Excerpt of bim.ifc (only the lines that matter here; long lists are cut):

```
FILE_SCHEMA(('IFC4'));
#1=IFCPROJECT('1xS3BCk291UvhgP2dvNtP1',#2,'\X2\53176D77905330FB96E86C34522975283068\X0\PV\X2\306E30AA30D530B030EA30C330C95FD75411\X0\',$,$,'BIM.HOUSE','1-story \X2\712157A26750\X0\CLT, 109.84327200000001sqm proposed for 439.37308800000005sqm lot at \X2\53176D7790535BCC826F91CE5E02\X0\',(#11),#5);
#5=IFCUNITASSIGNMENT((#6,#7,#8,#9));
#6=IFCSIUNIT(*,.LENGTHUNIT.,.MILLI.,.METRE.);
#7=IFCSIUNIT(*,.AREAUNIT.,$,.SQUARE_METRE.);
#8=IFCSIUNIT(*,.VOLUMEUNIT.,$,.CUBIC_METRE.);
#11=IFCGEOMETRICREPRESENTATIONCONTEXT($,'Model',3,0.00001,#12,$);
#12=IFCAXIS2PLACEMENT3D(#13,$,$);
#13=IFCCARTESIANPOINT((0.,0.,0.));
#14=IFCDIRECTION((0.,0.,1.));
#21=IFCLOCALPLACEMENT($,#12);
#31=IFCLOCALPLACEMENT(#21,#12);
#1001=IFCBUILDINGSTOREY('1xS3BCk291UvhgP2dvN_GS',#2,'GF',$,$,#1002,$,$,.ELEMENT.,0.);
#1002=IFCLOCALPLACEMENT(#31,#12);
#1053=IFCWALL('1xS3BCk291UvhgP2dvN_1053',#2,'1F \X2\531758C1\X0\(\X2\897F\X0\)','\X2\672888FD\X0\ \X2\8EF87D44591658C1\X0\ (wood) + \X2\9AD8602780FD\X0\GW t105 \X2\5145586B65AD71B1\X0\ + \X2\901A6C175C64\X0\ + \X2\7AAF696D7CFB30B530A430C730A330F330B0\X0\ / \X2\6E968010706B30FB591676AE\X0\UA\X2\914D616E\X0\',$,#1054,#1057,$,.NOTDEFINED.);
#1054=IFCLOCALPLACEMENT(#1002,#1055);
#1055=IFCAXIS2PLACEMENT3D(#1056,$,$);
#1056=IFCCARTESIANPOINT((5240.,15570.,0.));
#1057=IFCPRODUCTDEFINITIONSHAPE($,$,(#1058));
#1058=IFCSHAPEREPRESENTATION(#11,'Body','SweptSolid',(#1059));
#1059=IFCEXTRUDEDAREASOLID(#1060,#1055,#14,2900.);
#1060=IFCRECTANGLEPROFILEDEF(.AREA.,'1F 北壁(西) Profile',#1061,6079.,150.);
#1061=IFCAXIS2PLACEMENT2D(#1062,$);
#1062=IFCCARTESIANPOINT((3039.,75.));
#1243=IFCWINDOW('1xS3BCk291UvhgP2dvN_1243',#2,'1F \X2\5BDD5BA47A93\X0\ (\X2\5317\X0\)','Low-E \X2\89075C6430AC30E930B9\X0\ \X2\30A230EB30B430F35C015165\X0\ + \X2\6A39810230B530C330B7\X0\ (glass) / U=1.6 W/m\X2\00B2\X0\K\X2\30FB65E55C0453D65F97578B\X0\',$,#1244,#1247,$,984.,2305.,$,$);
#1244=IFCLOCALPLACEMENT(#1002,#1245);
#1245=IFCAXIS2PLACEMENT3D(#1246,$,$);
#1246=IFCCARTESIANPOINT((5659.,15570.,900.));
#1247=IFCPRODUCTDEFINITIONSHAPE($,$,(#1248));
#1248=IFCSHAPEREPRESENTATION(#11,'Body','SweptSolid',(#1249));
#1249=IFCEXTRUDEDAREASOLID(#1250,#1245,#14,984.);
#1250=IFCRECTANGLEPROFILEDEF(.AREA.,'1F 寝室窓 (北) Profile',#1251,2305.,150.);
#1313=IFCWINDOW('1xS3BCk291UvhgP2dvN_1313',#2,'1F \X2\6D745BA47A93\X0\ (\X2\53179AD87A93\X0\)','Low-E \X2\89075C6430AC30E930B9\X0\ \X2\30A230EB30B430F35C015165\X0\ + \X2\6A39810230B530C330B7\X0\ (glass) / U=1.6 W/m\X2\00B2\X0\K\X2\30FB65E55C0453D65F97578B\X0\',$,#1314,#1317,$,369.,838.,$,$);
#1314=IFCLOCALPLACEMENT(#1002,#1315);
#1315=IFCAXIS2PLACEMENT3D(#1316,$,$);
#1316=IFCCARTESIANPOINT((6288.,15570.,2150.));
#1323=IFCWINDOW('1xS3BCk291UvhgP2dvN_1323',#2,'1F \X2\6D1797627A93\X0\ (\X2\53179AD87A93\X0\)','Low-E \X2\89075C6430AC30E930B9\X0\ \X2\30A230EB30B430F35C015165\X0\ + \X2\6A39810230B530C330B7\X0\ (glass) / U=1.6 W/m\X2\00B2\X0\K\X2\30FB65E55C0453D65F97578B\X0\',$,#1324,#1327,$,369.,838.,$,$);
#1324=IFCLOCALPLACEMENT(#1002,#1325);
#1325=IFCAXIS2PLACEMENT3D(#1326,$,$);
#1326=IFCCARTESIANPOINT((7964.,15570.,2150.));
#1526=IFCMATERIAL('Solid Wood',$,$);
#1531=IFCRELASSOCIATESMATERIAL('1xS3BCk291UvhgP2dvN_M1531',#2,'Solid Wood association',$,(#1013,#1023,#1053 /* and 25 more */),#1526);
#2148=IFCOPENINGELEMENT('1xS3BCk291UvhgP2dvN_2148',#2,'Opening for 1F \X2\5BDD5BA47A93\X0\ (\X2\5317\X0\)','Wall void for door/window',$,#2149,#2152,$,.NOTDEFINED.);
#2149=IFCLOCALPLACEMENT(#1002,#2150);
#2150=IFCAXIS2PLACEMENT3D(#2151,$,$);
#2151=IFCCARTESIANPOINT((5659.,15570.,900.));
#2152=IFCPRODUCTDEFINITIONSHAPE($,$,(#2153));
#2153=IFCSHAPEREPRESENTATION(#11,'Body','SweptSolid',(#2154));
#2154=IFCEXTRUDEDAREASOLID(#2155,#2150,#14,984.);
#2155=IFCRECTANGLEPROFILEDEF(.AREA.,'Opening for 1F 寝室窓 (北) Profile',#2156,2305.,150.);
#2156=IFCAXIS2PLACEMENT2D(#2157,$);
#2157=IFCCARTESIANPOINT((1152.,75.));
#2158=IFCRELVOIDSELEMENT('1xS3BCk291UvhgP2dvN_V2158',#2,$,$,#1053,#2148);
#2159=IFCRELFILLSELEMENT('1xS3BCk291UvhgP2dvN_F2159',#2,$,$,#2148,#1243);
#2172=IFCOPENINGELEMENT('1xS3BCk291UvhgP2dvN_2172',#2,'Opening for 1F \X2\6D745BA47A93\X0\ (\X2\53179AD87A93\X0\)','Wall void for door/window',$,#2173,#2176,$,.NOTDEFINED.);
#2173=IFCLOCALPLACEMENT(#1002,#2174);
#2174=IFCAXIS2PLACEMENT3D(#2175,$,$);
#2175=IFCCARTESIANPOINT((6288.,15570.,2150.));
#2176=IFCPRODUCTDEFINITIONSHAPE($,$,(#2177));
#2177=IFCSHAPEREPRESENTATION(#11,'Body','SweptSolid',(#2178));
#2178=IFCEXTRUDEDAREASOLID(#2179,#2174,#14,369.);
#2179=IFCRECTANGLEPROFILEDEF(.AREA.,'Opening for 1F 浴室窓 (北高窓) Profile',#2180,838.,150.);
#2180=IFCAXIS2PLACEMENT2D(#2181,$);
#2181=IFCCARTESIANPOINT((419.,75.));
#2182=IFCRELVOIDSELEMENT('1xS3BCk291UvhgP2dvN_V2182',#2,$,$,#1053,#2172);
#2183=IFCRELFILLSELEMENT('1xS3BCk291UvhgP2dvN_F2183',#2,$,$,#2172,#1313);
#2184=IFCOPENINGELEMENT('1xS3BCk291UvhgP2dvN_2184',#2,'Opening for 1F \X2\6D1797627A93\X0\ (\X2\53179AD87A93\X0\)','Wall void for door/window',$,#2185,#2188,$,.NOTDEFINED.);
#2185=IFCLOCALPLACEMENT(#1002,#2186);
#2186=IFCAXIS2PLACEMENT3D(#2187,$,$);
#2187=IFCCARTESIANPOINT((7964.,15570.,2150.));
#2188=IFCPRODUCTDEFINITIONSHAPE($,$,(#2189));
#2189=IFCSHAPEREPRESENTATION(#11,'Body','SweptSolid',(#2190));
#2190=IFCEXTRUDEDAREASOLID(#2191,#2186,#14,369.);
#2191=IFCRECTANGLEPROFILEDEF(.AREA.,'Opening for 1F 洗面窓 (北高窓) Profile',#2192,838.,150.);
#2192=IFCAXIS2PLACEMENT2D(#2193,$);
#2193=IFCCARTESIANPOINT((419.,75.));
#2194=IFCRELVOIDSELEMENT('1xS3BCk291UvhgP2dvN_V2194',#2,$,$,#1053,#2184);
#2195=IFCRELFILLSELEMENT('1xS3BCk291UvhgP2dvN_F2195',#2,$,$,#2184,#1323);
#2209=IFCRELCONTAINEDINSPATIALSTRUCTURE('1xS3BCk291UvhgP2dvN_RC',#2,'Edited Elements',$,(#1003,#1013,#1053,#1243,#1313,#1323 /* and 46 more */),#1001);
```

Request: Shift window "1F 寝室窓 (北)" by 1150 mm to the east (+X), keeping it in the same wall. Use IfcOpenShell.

```python
import ifcopenshell
import ifcopenshell.api.geometry
import ifcopenshell.util.placement

model = ifcopenshell.open("bim.ifc")

window = model.by_guid("1xS3BCk291UvhgP2dvN_1243")
opening = window.FillsVoids[0].RelatingOpeningElement
wall = opening.VoidsElements[0].RelatingBuildingElement

wall_matrix = ifcopenshell.util.placement.get_local_placement(wall.ObjectPlacement)
shift = wall_matrix[:3, 0] * 1150.0
before = ifcopenshell.util.placement.get_local_placement(window.ObjectPlacement)[:3, 3].copy()

# The window is not placed relative to its opening, so move both.
for product in (opening, window):
    matrix = ifcopenshell.util.placement.get_local_placement(product.ObjectPlacement)
    matrix[:3, 3] += shift
    ifcopenshell.api.geometry.edit_object_placement(model, product=product, matrix=matrix, is_si=False)

after = ifcopenshell.util.placement.get_local_placement(window.ObjectPlacement)[:3, 3]
print("window moved by", (after - before).round(3) + 0.0)

model.write("bim_edited.ifc")
```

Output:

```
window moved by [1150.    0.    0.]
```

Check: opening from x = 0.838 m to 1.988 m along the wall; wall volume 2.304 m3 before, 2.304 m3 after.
